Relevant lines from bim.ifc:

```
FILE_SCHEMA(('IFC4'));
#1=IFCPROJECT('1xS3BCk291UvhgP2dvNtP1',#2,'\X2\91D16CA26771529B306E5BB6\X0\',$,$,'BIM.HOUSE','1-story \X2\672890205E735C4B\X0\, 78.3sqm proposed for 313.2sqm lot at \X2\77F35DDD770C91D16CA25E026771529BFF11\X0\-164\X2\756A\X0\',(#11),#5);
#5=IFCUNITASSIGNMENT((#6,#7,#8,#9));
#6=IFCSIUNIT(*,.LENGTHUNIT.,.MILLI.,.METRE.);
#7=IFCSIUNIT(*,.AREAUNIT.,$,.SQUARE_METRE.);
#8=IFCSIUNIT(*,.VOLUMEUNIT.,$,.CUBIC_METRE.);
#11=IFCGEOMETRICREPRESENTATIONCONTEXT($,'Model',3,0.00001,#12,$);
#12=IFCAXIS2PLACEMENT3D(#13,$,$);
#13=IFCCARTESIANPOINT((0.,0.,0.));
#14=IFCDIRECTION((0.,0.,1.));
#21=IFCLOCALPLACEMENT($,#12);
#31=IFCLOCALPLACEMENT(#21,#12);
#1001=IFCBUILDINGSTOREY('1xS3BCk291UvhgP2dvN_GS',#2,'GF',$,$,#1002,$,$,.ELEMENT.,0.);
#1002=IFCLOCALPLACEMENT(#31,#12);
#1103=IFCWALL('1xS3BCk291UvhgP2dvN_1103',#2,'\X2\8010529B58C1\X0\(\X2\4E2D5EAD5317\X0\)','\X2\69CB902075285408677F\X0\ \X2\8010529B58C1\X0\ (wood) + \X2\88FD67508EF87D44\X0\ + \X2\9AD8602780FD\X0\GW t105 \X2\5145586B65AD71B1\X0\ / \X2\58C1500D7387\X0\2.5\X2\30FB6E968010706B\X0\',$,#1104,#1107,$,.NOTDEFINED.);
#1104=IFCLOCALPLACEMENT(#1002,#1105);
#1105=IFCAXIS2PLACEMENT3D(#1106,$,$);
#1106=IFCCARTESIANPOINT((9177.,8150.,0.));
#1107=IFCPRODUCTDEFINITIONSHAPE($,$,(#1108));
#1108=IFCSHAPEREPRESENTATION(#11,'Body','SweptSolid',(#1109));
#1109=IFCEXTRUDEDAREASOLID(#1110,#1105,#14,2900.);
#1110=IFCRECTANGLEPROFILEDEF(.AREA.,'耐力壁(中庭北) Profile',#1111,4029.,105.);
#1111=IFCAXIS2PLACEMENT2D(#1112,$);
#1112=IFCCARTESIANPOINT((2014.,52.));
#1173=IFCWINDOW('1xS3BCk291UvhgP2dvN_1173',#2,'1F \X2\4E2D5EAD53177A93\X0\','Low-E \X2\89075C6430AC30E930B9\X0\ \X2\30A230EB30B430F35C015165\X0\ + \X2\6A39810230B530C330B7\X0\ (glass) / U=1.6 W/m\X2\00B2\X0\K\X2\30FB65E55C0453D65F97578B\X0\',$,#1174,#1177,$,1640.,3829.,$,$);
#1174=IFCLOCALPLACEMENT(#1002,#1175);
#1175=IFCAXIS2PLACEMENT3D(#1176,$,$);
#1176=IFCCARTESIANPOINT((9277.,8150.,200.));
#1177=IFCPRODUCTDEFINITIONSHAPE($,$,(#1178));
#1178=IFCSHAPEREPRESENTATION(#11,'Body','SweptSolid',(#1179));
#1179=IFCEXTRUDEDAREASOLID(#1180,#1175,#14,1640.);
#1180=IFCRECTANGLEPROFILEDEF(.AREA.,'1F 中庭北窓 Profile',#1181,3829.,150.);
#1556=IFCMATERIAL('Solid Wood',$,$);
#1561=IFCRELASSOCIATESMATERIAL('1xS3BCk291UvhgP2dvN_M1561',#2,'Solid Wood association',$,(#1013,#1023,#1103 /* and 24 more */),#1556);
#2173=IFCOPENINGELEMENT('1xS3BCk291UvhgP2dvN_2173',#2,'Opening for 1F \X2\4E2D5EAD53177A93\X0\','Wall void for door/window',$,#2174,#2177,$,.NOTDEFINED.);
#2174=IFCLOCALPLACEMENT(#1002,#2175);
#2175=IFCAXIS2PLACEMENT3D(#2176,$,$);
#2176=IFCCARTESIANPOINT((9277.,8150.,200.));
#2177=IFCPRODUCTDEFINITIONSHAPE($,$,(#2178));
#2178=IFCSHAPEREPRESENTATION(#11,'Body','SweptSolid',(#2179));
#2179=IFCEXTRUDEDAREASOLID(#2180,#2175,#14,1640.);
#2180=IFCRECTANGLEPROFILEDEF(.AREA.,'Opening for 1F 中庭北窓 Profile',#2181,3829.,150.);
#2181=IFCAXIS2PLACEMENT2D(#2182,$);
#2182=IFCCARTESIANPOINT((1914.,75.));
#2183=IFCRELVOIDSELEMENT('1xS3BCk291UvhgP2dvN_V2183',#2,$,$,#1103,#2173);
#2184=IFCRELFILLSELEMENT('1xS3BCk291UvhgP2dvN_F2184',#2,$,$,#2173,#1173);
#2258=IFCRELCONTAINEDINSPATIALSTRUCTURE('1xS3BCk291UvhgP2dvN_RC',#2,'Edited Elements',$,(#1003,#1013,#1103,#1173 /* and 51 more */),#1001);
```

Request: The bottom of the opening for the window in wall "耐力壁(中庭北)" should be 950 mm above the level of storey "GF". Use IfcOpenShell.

```python
import numpy as np
import ifcopenshell
import ifcopenshell.api.geometry
import ifcopenshell.geom
import ifcopenshell.util.element
import ifcopenshell.util.placement
import ifcopenshell.util.shape
import ifcopenshell.util.unit

model = ifcopenshell.open("bim.ifc")
unit_scale = ifcopenshell.util.unit.calculate_unit_scale(model)

window = model.by_guid("1xS3BCk291UvhgP2dvN_1173")
opening = window.FillsVoids[0].RelatingOpeningElement
storey = ifcopenshell.util.element.get_container(window, ifc_class="IfcBuildingStorey")
level = ifcopenshell.util.placement.get_local_placement(storey.ObjectPlacement)[2, 3]

# The opening's origin need not be at the sill, so measure its lowest point.
shape = ifcopenshell.geom.create_shape(ifcopenshell.geom.settings(), opening)
bottom = ifcopenshell.util.shape.get_shape_bottom_elevation(shape, shape.geometry) / unit_scale
dz = level + 0.95 / unit_scale - bottom

shift = np.array([0.0, 0.0, dz])
# The window is not placed relative to its opening, so move both.
for product in (opening, window):
    matrix = ifcopenshell.util.placement.get_local_placement(product.ObjectPlacement)
    matrix[:3, 3] += shift
    ifcopenshell.api.geometry.edit_object_placement(model, product=product, matrix=matrix, is_si=False)

print(f"moved by {dz * unit_scale:+.3f} m")

model.write("bim_v2.ifc")
```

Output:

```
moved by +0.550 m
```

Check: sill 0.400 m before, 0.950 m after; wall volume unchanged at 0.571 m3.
